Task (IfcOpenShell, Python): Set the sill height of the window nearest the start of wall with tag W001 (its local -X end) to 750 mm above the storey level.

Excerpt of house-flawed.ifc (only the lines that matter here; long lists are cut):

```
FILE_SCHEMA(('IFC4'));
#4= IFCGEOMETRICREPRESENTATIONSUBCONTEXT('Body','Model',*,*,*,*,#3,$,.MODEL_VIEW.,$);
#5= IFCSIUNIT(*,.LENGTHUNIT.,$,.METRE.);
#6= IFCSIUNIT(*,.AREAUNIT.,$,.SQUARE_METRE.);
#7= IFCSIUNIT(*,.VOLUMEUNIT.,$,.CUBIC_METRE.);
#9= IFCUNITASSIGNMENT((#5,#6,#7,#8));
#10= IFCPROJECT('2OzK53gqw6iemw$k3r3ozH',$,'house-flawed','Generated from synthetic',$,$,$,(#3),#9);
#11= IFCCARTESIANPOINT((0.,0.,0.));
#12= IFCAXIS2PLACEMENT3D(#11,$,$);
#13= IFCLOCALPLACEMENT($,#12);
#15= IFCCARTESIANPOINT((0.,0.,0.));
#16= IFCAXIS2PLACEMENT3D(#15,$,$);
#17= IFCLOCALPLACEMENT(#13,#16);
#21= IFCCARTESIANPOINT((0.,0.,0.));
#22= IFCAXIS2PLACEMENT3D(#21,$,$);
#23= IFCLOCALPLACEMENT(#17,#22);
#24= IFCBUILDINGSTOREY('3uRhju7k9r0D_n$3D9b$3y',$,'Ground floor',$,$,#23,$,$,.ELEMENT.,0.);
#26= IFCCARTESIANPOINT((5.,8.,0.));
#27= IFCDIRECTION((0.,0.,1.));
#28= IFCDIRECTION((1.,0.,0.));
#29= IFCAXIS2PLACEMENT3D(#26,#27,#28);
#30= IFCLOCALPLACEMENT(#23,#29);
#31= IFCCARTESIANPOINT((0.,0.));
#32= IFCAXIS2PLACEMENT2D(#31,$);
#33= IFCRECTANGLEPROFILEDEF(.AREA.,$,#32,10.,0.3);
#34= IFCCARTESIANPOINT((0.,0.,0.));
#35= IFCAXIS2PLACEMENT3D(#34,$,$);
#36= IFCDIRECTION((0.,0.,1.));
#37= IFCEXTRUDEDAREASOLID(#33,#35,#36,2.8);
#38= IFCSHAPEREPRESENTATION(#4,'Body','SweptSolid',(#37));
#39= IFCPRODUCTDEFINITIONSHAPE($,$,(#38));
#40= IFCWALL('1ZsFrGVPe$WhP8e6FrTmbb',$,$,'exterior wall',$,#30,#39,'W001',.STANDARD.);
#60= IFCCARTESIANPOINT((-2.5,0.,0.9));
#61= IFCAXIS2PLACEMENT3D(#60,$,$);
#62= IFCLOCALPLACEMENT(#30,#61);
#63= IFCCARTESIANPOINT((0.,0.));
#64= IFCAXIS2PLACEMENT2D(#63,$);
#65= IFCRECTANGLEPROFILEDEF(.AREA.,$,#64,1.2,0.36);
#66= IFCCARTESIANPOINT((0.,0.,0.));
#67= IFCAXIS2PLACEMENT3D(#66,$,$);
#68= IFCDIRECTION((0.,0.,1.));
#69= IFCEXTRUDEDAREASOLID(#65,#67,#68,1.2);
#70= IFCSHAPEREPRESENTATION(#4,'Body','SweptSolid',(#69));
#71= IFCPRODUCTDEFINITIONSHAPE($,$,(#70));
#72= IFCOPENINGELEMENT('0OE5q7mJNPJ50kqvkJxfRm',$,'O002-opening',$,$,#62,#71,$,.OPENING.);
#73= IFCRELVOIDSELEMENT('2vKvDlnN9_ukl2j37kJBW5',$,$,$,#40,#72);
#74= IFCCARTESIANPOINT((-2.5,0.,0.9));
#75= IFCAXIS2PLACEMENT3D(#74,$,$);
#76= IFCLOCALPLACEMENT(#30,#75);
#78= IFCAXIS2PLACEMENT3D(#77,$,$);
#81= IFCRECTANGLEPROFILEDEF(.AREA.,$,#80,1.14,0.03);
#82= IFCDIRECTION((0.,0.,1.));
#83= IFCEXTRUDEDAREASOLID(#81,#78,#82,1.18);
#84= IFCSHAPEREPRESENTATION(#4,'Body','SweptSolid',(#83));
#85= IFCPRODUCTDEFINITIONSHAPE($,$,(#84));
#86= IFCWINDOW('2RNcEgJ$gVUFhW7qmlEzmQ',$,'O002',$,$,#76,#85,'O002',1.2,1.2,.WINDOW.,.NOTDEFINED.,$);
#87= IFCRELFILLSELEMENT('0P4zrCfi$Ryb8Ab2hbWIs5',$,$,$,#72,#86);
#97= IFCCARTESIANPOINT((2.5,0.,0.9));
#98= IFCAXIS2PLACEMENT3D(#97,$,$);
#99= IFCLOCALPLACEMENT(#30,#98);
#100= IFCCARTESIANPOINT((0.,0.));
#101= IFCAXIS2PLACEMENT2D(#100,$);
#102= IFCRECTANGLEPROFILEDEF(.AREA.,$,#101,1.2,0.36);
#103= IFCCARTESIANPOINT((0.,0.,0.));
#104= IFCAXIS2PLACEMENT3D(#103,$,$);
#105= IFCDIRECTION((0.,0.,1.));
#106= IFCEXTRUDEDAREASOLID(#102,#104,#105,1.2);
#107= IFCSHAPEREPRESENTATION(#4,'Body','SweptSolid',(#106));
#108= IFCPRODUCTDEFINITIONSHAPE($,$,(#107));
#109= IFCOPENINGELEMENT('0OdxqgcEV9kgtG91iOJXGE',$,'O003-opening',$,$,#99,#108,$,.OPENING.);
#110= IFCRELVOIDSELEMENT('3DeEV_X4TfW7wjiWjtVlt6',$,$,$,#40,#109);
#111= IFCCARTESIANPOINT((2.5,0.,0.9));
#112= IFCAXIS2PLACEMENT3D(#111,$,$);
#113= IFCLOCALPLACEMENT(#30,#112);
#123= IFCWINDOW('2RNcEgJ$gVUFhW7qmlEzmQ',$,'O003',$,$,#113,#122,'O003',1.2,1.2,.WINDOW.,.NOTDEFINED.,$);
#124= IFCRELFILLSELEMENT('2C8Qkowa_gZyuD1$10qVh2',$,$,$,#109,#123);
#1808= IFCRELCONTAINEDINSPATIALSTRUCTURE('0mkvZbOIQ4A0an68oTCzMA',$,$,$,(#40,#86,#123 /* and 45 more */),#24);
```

```python
import numpy as np
import ifcopenshell
import ifcopenshell.api.geometry
import ifcopenshell.geom
import ifcopenshell.util.element
import ifcopenshell.util.placement
import ifcopenshell.util.shape
import ifcopenshell.util.unit

model = ifcopenshell.open("house-flawed.ifc")
unit_scale = ifcopenshell.util.unit.calculate_unit_scale(model)

window = model.by_id(86)
opening = window.FillsVoids[0].RelatingOpeningElement
storey = ifcopenshell.util.element.get_container(window, ifc_class="IfcBuildingStorey")
level = ifcopenshell.util.placement.get_local_placement(storey.ObjectPlacement)[2, 3]

# The opening's origin need not be at the sill, so measure its lowest point.
shape = ifcopenshell.geom.create_shape(ifcopenshell.geom.settings(), opening)
bottom = ifcopenshell.util.shape.get_shape_bottom_elevation(shape, shape.geometry) / unit_scale
dz = level + 0.75 / unit_scale - bottom

shift = np.array([0.0, 0.0, dz])
# The window is not placed relative to its opening, so move both.
for product in (opening, window):
    matrix = ifcopenshell.util.placement.get_local_placement(product.ObjectPlacement)
    matrix[:3, 3] += shift
    ifcopenshell.api.geometry.edit_object_placement(model, product=product, matrix=matrix, is_si=False)

print(f"moved by {dz * unit_scale:+.3f} m")

model.write("house-flawed_v2.ifc")
```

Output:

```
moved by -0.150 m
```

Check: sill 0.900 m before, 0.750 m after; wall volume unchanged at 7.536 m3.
